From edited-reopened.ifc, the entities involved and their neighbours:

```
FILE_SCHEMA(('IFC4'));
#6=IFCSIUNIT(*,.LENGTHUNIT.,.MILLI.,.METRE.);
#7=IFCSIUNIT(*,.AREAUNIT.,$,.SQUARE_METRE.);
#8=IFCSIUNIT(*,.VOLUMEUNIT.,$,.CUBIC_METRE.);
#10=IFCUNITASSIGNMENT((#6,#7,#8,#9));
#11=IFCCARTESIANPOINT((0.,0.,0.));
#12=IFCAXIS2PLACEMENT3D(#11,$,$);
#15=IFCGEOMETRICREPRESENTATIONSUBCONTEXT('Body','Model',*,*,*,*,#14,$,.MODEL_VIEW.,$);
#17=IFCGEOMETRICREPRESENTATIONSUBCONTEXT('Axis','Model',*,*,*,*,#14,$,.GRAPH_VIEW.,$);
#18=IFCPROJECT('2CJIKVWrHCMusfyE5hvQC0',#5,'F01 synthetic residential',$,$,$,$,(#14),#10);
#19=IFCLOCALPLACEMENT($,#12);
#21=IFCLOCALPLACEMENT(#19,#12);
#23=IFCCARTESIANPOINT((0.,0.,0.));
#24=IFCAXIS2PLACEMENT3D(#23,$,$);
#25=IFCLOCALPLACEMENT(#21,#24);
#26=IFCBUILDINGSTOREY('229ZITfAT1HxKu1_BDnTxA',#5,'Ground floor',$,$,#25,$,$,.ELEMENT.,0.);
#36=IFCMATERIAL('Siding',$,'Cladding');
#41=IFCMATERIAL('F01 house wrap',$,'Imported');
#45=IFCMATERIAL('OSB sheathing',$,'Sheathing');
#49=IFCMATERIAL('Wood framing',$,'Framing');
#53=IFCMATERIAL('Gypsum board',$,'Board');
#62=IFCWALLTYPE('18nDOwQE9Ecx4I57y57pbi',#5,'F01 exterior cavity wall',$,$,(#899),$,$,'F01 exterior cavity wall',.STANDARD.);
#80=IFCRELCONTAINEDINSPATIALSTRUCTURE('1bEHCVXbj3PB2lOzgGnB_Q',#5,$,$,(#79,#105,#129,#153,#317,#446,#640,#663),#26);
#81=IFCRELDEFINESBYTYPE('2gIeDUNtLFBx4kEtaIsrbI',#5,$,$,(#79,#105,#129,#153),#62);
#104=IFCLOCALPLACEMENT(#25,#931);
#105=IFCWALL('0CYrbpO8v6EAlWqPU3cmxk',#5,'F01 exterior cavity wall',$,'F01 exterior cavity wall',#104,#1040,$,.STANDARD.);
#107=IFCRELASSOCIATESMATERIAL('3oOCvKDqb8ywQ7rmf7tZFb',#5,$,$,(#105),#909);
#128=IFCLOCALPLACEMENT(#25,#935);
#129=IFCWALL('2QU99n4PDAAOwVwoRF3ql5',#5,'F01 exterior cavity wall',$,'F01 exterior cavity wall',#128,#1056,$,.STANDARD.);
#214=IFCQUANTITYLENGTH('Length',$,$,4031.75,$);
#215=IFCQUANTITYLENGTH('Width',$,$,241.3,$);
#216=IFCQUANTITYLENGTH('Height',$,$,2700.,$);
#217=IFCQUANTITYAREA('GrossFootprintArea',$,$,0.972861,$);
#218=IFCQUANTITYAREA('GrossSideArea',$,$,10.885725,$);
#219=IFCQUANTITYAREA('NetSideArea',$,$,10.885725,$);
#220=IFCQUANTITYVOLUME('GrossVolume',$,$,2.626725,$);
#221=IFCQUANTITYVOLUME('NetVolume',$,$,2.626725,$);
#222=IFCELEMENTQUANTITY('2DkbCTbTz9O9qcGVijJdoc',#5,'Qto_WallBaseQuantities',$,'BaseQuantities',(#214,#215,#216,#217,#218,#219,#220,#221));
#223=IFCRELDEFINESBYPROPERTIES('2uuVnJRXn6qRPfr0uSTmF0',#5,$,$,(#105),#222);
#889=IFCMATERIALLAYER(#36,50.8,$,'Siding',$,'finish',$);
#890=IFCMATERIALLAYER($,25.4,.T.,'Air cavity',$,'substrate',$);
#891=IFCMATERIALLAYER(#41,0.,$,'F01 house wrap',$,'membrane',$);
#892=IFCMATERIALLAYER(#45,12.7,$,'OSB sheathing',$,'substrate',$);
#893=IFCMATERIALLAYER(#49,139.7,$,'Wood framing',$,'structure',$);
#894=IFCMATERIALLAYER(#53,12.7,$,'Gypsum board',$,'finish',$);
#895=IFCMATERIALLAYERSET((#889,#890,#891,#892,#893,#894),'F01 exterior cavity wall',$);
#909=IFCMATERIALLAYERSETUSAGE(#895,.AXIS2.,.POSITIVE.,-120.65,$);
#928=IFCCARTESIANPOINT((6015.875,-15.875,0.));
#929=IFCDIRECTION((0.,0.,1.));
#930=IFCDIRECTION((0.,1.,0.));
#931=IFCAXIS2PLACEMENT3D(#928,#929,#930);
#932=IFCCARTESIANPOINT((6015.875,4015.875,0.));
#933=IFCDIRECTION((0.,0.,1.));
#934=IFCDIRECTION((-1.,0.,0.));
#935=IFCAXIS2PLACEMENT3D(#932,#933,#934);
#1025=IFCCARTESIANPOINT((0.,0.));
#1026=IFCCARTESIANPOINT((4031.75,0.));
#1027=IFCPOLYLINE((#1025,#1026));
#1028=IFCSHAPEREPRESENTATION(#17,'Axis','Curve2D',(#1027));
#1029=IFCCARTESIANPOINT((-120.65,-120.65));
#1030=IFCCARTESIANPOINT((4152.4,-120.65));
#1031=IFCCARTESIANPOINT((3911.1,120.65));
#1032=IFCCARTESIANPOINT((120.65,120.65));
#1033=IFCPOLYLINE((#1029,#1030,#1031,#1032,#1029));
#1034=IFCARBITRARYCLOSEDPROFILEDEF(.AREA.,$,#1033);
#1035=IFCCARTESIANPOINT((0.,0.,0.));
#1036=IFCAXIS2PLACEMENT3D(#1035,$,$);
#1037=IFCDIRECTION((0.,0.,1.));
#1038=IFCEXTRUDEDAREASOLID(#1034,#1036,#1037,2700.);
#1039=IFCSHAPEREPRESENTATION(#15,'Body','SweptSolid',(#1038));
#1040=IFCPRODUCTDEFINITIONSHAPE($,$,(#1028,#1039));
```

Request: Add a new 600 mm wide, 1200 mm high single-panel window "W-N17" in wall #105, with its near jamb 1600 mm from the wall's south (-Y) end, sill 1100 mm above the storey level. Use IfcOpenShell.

```python
import numpy as np
import ifcopenshell
import ifcopenshell.api.feature
import ifcopenshell.api.geometry
import ifcopenshell.api.pset
import ifcopenshell.api.root
import ifcopenshell.api.spatial
import ifcopenshell.geom
import ifcopenshell.util.element
import ifcopenshell.util.placement
import ifcopenshell.util.representation
import ifcopenshell.util.shape
import ifcopenshell.util.unit

model = ifcopenshell.open("edited-reopened.ifc")
unit_scale = ifcopenshell.util.unit.calculate_unit_scale(model)
area_scale = ifcopenshell.util.unit.calculate_unit_scale(model, "AREAUNIT")
volume_scale = ifcopenshell.util.unit.calculate_unit_scale(model, "VOLUMEUNIT")
settings = ifcopenshell.geom.settings()


def volume(element):
    """Net volume in cubic metres, openings subtracted."""
    shape = ifcopenshell.geom.create_shape(settings, element)
    return ifcopenshell.util.shape.get_volume(shape.geometry)


wall = model.by_guid("0CYrbpO8v6EAlWqPU3cmxk")
storey = ifcopenshell.util.element.get_container(wall, ifc_class="IfcBuildingStorey")
context = ifcopenshell.util.representation.get_context(model, "Model", "Body", "MODEL_VIEW")
before = volume(wall)

width, height, from_end, sill = 0.6, 1.2, 1.6, 1.1  # metres

# The wall runs along its own X axis, and the end named is its -X end.
wall_shape = ifcopenshell.geom.create_shape(settings, wall)
x, y, z = ifcopenshell.util.shape.get_vertices(wall_shape.geometry).T
start = x.min() + from_end
face, thickness = float(y.min()), float(y.max() - y.min())
wall_matrix = ifcopenshell.util.placement.get_local_placement(wall.ObjectPlacement)
level = ifcopenshell.util.placement.get_local_placement(storey.ObjectPlacement)[2, 3]


def in_wall(x, y):
    """Placement at x, y metres in the wall's axes, at sill height."""
    matrix = wall_matrix.copy()
    matrix[:, 3] = wall_matrix @ np.array([x / unit_scale, y / unit_scale, 0.0, 1.0])
    matrix[2, 3] = level + sill / unit_scale
    return matrix


# Opening: a box that overshoots both wall faces by 50 mm.
opening = ifcopenshell.api.root.create_entity(model, ifc_class="IfcOpeningElement", predefined_type="OPENING")
box = ifcopenshell.api.geometry.add_wall_representation(
    model, context=context, length=width, height=height, thickness=thickness + 0.1
)
ifcopenshell.api.geometry.assign_representation(model, product=opening, representation=box)
ifcopenshell.api.geometry.edit_object_placement(model, product=opening, matrix=in_wall(start, face - 0.05), is_si=False)
ifcopenshell.api.feature.add_feature(model, feature=opening, element=wall)

window = ifcopenshell.api.root.create_entity(model, ifc_class="IfcWindow", name="W-N17", predefined_type="WINDOW")
window.OverallWidth, window.OverallHeight = width / unit_scale, height / unit_scale
window.PartitioningType = "SINGLE_PANEL"
body = ifcopenshell.api.geometry.add_window_representation(
    model,
    context=context,
    overall_width=window.OverallWidth,
    overall_height=window.OverallHeight,
    partition_type="SINGLE_PANEL",
)
ifcopenshell.api.geometry.assign_representation(model, product=window, representation=body)
ifcopenshell.api.spatial.assign_container(model, products=[window], relating_structure=storey)
ifcopenshell.api.feature.add_filling(model, opening=opening, element=window)

# Centre the window in the wall's thickness.
ifcopenshell.api.geometry.edit_object_placement(model, product=window, matrix=in_wall(start, face), is_si=False)
window_shape = ifcopenshell.geom.create_shape(settings, window)
depth = ifcopenshell.util.shape.get_vertices(window_shape.geometry)[:, 1]
offset = face + thickness / 2 - (depth.min() + depth.max()) / 2
ifcopenshell.api.geometry.edit_object_placement(model, product=window, matrix=in_wall(start, offset), is_si=False)

after = volume(wall)

# Update the wall's stored quantities.
qto = model.by_id(ifcopenshell.util.element.get_pset(wall, "Qto_WallBaseQuantities", should_inherit=False)["id"])
ifcopenshell.api.pset.edit_qto(model, qto=qto, properties={
    "NetSideArea": after / thickness / area_scale,
    "NetVolume": after / volume_scale,
})

print(f"wall volume {before:.3f} -> {after:.3f} m3")

model.write("edited-reopened_edited.ifc")
```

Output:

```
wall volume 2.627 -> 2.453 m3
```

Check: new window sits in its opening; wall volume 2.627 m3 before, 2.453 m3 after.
